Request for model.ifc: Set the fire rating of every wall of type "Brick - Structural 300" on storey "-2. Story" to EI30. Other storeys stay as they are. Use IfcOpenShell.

First a look at what the model holds.

```python
import ifcopenshell
import ifcopenshell.util.element

model = ifcopenshell.open("model.ifc")
print(model.schema)
storey = next(s for s in model.by_type("IfcBuildingStorey") if s.Name == "-2. Story")
walls = [e for e in ifcopenshell.util.element.get_decomposition(storey) if e.is_a("IfcWall")]
seen = {}
for e in walls:
    element_type = ifcopenshell.util.element.get_type(e)
    key = (element_type.Name if element_type != e and element_type else None, ifcopenshell.util.element.get_pset(e, "Pset_WallCommon", "FireRating"))
    seen[key] = seen.get(key, 0) + 1
for (name, value), count in sorted(seen.items(), key=str):
    print(count, "x", name, "|", value)
```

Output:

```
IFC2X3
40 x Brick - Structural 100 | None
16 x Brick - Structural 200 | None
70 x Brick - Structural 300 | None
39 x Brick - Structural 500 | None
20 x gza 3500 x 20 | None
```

```python
import ifcopenshell
import ifcopenshell.api.pset
import ifcopenshell.util.element

model = ifcopenshell.open("model.ifc")

storey = next(s for s in model.by_type("IfcBuildingStorey") if s.Name == "-2. Story")
walls = [e for e in ifcopenshell.util.element.get_decomposition(storey) if e.is_a("IfcWall")]

count = 0
for e in walls:
    element_type = ifcopenshell.util.element.get_type(e)
    if element_type in (None, e) or element_type.Name != "Brick - Structural 300":
        continue
    # add_pset returns the element's existing set when there is one.
    pset = ifcopenshell.api.pset.add_pset(model, product=e, name="Pset_WallCommon")
    ifcopenshell.api.pset.edit_pset(model, pset=pset, properties={"FireRating": "EI30"})
    count += 1

print(count, "walls updated")

model.write("model_updated.ifc")
```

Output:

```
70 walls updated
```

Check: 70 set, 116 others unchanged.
